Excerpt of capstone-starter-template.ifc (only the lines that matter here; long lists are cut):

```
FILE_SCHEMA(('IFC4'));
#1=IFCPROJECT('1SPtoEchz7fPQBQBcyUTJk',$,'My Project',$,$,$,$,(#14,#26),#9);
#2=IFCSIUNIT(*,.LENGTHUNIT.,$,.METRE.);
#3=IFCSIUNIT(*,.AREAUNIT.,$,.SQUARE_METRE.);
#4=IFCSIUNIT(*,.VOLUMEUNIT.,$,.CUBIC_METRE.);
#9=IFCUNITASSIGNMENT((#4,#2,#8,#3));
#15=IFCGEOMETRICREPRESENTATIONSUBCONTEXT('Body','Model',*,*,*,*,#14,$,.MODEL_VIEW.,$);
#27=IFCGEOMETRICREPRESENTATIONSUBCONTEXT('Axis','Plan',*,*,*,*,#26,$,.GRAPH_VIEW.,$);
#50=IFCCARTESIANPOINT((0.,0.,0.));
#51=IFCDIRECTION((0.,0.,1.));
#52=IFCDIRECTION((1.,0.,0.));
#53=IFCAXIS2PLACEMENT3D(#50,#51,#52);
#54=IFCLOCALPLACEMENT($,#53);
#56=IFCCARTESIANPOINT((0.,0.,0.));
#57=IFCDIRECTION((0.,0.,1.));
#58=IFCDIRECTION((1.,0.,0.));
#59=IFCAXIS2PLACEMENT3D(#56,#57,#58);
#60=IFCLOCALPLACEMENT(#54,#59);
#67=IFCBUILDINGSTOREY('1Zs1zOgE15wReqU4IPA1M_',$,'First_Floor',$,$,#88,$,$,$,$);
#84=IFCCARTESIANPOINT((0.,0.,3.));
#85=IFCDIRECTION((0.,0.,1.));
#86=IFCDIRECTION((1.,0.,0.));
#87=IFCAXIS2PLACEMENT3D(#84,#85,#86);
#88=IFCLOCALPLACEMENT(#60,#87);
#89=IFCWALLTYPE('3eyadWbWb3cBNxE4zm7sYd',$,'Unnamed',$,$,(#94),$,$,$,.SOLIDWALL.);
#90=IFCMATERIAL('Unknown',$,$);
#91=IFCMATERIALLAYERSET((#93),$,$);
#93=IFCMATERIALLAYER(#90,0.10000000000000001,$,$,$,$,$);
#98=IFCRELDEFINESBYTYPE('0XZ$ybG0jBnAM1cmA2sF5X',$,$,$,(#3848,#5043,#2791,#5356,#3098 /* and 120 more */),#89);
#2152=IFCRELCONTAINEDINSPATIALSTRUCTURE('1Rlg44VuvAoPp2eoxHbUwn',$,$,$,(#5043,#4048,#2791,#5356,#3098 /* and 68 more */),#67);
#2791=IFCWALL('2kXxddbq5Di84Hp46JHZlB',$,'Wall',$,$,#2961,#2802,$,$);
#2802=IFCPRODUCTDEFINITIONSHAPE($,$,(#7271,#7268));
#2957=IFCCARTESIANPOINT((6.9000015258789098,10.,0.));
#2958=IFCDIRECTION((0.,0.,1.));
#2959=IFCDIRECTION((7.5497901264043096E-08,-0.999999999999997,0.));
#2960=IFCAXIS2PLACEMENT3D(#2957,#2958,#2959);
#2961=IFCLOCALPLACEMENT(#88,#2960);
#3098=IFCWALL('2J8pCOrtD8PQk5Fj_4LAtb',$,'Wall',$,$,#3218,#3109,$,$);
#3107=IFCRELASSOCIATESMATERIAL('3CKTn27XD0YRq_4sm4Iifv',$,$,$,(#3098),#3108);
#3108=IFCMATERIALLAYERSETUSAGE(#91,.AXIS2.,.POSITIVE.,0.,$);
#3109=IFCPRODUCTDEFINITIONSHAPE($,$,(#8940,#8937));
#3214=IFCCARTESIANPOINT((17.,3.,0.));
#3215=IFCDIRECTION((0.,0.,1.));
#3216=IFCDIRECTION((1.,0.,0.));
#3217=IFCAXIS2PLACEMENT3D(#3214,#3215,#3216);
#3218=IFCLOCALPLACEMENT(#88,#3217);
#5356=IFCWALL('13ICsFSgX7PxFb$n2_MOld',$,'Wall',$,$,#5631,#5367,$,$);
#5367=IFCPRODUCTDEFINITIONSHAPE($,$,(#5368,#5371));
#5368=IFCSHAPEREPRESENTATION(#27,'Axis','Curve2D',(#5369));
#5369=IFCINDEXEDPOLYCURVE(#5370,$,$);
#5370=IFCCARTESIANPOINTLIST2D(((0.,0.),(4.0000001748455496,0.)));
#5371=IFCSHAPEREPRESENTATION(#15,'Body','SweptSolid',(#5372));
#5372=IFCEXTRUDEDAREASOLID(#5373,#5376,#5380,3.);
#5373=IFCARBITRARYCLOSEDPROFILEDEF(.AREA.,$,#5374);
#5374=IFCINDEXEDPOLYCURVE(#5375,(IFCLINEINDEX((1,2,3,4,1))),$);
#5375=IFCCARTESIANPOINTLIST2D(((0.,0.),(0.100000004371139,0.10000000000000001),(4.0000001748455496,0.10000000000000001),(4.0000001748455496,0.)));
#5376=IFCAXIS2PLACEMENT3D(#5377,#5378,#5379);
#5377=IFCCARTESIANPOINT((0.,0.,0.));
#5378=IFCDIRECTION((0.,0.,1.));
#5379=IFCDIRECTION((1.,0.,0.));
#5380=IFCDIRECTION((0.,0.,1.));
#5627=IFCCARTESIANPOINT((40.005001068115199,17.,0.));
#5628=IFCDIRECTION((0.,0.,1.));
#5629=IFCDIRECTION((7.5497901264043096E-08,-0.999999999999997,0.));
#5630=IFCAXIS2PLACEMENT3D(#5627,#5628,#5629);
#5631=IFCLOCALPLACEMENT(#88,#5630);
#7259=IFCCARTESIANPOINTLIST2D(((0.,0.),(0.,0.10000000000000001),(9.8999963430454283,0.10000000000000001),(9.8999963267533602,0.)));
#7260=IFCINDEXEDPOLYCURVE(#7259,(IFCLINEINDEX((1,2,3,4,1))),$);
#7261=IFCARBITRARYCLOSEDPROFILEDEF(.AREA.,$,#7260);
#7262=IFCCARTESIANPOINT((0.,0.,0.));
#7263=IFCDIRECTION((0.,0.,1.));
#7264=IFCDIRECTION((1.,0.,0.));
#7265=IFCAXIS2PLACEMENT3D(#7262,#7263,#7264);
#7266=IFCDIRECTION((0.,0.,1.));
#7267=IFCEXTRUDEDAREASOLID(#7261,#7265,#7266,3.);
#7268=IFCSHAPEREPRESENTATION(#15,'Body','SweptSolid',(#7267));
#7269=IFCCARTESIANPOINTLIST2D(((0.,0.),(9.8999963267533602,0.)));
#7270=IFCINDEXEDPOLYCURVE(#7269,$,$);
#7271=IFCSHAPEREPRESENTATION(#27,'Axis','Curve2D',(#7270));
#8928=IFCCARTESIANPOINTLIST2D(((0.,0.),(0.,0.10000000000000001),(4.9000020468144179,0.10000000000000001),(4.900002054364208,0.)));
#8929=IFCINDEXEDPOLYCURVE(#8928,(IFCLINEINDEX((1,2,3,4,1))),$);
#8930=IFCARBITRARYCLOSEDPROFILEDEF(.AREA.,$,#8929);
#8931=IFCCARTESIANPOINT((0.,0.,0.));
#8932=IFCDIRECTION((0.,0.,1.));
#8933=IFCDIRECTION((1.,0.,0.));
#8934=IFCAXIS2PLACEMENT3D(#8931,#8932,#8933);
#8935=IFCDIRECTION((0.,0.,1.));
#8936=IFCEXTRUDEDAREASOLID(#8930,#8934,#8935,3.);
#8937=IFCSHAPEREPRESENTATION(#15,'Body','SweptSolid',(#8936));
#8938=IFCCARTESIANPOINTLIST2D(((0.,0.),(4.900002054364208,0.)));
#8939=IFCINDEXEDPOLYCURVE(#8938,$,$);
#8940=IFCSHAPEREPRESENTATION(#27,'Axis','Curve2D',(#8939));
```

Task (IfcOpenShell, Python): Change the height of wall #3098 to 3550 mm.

```python
import ifcopenshell
import ifcopenshell.geom
import ifcopenshell.util.representation
import ifcopenshell.util.shape

model = ifcopenshell.open("capstone-starter-template.ifc")
settings = ifcopenshell.geom.settings()


def volume(element):
    """Net volume in cubic metres, openings subtracted."""
    shape = ifcopenshell.geom.create_shape(settings, element)
    return ifcopenshell.util.shape.get_volume(shape.geometry)


wall = model.by_guid("2J8pCOrtD8PQk5Fj_4LAtb")
before = volume(wall)

body = ifcopenshell.util.representation.get_representation(wall, "Model", "Body")
solid = body.Items[0]
old_height = solid.Depth
solid.Depth = 3.55
after = volume(wall)

print(f"height {old_height:g} -> {solid.Depth:g}, volume {before:.3f} -> {after:.3f} m3")

model.write("capstone-starter-template_v2.ifc")
```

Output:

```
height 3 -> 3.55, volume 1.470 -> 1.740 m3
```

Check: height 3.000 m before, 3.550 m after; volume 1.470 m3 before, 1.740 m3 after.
